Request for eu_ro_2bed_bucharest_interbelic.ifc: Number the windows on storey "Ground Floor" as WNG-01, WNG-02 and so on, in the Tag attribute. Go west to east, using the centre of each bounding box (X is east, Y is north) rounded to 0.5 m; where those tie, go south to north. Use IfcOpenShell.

First a look at what the model holds.

```python
import ifcopenshell
import ifcopenshell.util.element
import ifcopenshell.util.placement

model = ifcopenshell.open("eu_ro_2bed_bucharest_interbelic.ifc")
print(model.schema)
storey = next(s for s in model.by_type("IfcBuildingStorey") if s.Name == "Ground Floor")
windows = [e for e in ifcopenshell.util.element.get_decomposition(storey) if e.is_a("IfcWindow")]
for e in sorted(windows, key=lambda e: e.id()):
    origin = ifcopenshell.util.placement.get_local_placement(e.ObjectPlacement)[:3, 3]
    print(e.id(), e.Tag, e.Name, origin.round(2) + 0.0, sep=" | ")
```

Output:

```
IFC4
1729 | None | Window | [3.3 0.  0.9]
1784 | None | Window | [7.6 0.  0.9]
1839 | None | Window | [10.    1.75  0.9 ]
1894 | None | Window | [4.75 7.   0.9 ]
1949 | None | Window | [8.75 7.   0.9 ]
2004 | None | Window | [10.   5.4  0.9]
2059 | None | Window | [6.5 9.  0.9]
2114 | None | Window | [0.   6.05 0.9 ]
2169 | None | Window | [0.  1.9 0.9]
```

```python
import ifcopenshell
import ifcopenshell.geom
import ifcopenshell.util.element
import ifcopenshell.util.shape

model = ifcopenshell.open("eu_ro_2bed_bucharest_interbelic.ifc")
settings = ifcopenshell.geom.settings()
settings.set("use-world-coords", True)


def centre(element):
    shape = ifcopenshell.geom.create_shape(settings, element)
    return ifcopenshell.util.shape.get_bbox_centroid(shape.geometry)


storey = next(s for s in model.by_type("IfcBuildingStorey") if s.Name == "Ground Floor")
windows = [e for e in ifcopenshell.util.element.get_decomposition(storey) if e.is_a("IfcWindow")]

# Insertion points can sit at a corner or the storey origin, so sort by the geometry (in metres).
centres = {e: centre(e) for e in windows}
windows.sort(key=lambda e: (round(centres[e][0] / 0.5), centres[e][1]))

for i, e in enumerate(windows, start=1):
    number = f"WNG-{i:02d}"
    e.Tag = number
    print(e.id(), number)

model.write("eu_ro_2bed_bucharest_interbelic-out.ifc")
```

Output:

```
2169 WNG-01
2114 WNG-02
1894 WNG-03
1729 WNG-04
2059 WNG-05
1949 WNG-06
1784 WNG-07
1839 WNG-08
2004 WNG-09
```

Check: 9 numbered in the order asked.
